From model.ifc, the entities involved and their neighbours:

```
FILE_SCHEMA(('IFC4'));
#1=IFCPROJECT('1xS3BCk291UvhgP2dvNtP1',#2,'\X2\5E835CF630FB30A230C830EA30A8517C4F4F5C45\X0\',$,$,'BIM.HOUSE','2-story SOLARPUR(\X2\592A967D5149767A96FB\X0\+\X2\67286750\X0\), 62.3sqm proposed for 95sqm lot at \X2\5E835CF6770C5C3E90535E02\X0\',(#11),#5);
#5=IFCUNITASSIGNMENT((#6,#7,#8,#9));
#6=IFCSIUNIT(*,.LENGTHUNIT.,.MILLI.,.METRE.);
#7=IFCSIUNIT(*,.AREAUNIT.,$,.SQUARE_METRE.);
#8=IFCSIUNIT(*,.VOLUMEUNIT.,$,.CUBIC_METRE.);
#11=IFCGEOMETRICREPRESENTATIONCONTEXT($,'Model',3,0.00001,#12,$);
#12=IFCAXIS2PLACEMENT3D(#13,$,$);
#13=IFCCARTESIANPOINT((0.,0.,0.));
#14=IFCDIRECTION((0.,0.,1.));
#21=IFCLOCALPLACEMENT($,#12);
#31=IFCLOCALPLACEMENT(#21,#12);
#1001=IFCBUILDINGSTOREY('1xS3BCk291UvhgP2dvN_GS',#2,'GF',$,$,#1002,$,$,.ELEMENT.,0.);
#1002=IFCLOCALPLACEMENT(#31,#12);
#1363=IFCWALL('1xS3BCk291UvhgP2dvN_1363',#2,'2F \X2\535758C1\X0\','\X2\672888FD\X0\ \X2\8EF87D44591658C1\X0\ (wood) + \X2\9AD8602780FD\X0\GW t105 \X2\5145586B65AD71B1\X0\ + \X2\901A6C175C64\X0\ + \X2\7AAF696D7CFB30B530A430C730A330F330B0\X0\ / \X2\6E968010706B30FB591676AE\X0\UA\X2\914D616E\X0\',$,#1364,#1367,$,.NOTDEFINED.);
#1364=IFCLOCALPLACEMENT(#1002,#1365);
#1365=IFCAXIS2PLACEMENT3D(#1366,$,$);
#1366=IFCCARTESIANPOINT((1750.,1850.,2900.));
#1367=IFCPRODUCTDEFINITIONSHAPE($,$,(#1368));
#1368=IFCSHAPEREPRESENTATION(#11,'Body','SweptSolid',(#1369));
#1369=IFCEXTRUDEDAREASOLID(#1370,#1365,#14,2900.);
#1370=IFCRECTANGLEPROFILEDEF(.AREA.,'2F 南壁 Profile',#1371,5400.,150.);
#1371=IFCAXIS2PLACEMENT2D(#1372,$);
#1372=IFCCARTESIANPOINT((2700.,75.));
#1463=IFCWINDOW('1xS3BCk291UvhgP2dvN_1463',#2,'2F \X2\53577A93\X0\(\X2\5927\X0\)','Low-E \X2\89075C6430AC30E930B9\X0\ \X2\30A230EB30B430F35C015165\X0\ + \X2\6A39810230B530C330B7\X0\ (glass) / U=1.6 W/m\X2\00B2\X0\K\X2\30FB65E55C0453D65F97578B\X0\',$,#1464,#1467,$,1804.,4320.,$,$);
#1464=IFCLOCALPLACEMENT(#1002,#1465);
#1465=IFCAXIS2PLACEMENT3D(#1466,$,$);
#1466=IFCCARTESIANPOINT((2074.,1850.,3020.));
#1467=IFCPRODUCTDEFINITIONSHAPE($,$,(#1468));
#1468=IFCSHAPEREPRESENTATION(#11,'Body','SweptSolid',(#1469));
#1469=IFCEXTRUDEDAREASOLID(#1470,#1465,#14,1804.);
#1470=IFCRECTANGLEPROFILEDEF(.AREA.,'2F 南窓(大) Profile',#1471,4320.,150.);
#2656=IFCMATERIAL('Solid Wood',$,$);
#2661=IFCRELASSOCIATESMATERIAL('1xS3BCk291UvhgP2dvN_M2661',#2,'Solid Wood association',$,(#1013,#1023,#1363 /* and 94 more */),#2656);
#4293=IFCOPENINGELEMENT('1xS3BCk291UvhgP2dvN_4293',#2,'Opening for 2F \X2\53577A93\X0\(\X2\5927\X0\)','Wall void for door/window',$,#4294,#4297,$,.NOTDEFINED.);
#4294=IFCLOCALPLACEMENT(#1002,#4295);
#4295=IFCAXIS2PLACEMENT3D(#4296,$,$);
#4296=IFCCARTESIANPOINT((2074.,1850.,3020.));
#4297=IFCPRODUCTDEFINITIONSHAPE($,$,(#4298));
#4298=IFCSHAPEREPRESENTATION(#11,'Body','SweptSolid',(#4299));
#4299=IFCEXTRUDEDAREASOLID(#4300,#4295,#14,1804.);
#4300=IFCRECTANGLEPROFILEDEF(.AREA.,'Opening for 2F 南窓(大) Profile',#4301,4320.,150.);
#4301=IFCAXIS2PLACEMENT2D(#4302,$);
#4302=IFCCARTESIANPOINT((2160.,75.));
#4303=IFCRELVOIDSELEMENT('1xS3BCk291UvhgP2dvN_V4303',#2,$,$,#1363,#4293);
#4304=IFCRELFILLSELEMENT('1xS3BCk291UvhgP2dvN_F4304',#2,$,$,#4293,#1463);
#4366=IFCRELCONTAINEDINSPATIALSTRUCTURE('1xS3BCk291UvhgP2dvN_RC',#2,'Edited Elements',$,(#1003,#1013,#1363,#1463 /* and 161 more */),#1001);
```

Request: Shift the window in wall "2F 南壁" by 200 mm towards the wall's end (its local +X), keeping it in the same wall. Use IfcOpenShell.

```python
import ifcopenshell
import ifcopenshell.api.geometry
import ifcopenshell.util.placement
import ifcopenshell.util.unit

model = ifcopenshell.open("model.ifc")
unit_scale = ifcopenshell.util.unit.calculate_unit_scale(model)

window = model.by_guid("1xS3BCk291UvhgP2dvN_1463")
opening = window.FillsVoids[0].RelatingOpeningElement
wall = opening.VoidsElements[0].RelatingBuildingElement

wall_matrix = ifcopenshell.util.placement.get_local_placement(wall.ObjectPlacement)
shift = wall_matrix[:3, 0] * 0.2 / unit_scale
before = ifcopenshell.util.placement.get_local_placement(window.ObjectPlacement)[:3, 3].copy()

# The window is not placed relative to its opening, so move both.
for product in (opening, window):
    matrix = ifcopenshell.util.placement.get_local_placement(product.ObjectPlacement)
    matrix[:3, 3] += shift
    ifcopenshell.api.geometry.edit_object_placement(model, product=product, matrix=matrix, is_si=False)

after = ifcopenshell.util.placement.get_local_placement(window.ObjectPlacement)[:3, 3]
print("window moved by", (after - before).round(3) + 0.0)

model.write("model_edited.ifc")
```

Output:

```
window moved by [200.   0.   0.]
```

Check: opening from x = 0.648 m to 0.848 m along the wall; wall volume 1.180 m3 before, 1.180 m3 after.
